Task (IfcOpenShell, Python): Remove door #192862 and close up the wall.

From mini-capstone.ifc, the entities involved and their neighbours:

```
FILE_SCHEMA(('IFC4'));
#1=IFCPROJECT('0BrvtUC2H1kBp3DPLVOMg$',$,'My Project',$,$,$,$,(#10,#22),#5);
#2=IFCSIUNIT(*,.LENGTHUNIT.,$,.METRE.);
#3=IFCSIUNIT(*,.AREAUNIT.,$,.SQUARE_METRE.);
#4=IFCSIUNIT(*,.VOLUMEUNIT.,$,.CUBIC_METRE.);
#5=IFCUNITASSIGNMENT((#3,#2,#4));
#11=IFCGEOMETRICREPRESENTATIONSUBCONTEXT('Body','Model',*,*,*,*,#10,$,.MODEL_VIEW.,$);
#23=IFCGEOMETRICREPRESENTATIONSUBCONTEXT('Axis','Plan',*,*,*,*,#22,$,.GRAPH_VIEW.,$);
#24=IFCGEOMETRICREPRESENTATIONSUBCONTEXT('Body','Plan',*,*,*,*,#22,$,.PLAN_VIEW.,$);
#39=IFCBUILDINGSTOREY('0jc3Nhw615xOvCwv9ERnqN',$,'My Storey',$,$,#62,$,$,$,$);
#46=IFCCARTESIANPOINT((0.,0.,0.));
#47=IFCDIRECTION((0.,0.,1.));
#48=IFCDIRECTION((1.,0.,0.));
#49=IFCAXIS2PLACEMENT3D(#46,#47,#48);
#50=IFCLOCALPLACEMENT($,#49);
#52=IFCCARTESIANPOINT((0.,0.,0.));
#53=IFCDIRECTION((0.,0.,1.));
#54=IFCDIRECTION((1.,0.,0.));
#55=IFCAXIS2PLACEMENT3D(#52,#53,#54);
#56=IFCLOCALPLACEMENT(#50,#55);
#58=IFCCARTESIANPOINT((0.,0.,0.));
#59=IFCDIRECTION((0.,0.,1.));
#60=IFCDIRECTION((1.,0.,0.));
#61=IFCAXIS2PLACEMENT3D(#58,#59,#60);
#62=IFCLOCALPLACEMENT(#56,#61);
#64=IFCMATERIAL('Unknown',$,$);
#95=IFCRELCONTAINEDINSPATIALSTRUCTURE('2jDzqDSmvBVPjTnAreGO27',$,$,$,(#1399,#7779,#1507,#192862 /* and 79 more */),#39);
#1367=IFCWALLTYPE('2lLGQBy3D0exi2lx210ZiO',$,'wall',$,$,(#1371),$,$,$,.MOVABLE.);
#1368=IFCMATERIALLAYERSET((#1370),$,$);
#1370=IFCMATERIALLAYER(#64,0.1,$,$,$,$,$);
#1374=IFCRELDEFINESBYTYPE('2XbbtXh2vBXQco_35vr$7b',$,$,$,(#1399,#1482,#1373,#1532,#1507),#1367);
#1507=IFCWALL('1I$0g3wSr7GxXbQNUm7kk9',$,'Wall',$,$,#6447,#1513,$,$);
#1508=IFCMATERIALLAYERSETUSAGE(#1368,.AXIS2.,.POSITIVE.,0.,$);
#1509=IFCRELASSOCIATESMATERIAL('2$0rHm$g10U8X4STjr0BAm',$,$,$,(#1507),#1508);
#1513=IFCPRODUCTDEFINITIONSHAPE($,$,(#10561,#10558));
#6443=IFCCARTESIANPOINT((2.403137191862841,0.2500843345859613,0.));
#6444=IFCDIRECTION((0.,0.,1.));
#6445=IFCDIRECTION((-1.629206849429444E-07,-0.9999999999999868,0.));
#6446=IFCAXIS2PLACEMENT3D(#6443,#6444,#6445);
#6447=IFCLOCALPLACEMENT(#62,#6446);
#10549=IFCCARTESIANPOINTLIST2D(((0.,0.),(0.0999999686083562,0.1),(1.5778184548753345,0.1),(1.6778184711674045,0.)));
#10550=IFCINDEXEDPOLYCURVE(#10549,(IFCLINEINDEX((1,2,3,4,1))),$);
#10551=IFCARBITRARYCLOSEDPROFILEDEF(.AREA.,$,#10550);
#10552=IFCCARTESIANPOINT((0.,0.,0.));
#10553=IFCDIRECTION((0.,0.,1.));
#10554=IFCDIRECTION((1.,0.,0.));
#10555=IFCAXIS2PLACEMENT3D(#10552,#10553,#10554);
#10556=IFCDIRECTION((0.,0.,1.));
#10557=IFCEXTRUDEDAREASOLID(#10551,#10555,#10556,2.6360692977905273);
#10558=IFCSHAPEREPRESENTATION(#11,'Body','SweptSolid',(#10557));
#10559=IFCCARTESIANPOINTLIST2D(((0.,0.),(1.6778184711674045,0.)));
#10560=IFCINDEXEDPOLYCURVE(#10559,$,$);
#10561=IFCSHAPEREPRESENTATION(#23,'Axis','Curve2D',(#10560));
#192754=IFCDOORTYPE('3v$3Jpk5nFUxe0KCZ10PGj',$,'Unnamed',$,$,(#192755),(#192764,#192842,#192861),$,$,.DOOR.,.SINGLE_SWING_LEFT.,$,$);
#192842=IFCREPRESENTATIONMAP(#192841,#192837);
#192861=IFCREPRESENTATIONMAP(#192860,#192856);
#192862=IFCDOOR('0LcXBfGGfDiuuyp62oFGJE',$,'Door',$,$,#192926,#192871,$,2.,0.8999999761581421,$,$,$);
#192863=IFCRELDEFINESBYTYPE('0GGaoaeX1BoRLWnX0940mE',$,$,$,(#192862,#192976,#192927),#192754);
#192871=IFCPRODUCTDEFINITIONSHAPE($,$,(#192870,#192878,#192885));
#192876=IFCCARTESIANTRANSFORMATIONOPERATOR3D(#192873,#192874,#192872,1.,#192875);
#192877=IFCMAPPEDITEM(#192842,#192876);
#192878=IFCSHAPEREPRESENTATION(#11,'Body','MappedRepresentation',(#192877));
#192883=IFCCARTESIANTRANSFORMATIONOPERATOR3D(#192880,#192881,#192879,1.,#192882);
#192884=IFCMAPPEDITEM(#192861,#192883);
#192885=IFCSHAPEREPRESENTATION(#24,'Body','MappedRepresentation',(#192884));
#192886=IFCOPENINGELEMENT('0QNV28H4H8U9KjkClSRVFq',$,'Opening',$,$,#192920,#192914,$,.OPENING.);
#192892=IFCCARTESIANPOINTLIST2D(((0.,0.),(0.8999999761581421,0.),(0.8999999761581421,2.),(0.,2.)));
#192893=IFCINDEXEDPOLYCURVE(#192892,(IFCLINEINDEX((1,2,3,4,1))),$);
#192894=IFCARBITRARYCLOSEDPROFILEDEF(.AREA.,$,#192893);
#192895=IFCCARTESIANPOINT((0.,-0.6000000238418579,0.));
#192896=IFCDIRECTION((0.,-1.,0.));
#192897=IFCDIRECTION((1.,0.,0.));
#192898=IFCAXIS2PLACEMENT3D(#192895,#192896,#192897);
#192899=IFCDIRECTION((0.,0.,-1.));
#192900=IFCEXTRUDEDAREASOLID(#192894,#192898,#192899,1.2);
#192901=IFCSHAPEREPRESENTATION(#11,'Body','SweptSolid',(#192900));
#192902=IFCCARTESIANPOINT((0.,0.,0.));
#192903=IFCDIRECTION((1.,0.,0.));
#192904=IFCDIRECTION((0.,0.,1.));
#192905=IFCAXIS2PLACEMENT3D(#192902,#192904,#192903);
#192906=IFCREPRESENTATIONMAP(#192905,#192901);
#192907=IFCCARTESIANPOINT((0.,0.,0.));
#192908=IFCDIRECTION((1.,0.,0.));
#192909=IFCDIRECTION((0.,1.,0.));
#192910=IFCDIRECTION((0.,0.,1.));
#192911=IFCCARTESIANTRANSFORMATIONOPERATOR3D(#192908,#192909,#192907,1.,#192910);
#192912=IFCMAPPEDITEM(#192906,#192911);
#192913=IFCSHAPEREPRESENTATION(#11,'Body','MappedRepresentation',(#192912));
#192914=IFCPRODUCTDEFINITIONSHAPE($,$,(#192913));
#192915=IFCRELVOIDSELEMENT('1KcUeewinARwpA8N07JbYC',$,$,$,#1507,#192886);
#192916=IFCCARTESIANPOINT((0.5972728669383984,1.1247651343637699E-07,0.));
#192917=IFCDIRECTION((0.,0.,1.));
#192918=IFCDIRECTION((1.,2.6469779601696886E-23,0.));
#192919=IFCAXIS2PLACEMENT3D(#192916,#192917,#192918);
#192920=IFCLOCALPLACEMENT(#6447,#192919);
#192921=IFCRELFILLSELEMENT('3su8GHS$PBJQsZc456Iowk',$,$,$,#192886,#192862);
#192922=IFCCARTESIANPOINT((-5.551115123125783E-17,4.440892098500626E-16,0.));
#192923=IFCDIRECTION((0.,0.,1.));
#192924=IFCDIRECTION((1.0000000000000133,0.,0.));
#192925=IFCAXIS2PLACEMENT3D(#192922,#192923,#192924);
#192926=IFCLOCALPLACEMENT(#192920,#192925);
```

```python
import ifcopenshell
import ifcopenshell.api.feature
import ifcopenshell.api.root
import ifcopenshell.geom
import ifcopenshell.util.shape

model = ifcopenshell.open("mini-capstone.ifc")
settings = ifcopenshell.geom.settings()


def volume(element):
    """Net volume in cubic metres, openings subtracted."""
    shape = ifcopenshell.geom.create_shape(settings, element)
    return ifcopenshell.util.shape.get_volume(shape.geometry)


door = model.by_id(192862)
opening = door.FillsVoids[0].RelatingOpeningElement
wall = opening.VoidsElements[0].RelatingBuildingElement
before = volume(wall)

ifcopenshell.api.root.remove_product(model, product=door)
ifcopenshell.api.feature.remove_feature(model, feature=opening)

after = volume(wall)

print(f"wall volume {before:.3f} -> {after:.3f} m3")

model.write("mini-capstone-out.ifc")
```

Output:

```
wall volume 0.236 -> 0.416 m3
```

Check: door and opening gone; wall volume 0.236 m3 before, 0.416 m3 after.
